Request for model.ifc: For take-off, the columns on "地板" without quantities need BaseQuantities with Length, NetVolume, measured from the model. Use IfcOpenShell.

First a look at what the model holds.

```python
import ifcopenshell
import ifcopenshell.util.element
import ifcopenshell.util.unit

model = ifcopenshell.open("model.ifc")
print(model.schema)
for unit_type in ("LENGTHUNIT", "AREAUNIT", "VOLUMEUNIT"):
    print(unit_type, ifcopenshell.util.unit.calculate_unit_scale(model, unit_type))
storey = next(s for s in model.by_type("IfcBuildingStorey") if s.Name == "地板")
columns = [e for e in ifcopenshell.util.element.get_decomposition(storey) if e.is_a("IfcColumn")]
for e in sorted(columns, key=lambda e: e.id()):
    print(e.id(), e.is_a(), e.Name, list(ifcopenshell.util.element.get_psets(e, qtos_only=True)), sep=" | ")
```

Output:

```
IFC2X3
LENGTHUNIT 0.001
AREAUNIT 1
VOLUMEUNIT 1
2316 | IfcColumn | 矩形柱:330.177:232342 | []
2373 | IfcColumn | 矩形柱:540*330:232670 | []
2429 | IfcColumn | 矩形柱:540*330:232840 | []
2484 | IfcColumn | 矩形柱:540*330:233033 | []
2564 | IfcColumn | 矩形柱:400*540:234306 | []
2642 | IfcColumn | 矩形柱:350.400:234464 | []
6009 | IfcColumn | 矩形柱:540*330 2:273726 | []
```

```python
import ifcopenshell
import ifcopenshell.api.pset
import ifcopenshell.geom
import ifcopenshell.util.element
import ifcopenshell.util.shape
import ifcopenshell.util.unit

model = ifcopenshell.open("model.ifc")
unit_scale = ifcopenshell.util.unit.calculate_unit_scale(model)
volume_scale = ifcopenshell.util.unit.calculate_unit_scale(model, "VOLUMEUNIT")
settings = ifcopenshell.geom.settings()

storey = next(s for s in model.by_type("IfcBuildingStorey") if s.Name == "地板")
columns = [e for e in ifcopenshell.util.element.get_decomposition(storey) if e.is_a("IfcColumn")]

for e in sorted(columns, key=lambda e: e.id()):
    if ifcopenshell.util.element.get_psets(e, qtos_only=True, should_inherit=False):
        continue
    # Geometry comes back in metres, in the element's own axes.
    shape = ifcopenshell.geom.create_shape(settings, e)
    values = {
        "Length": ifcopenshell.util.shape.get_z(shape.geometry) / unit_scale,
        "NetVolume": ifcopenshell.util.shape.get_volume(shape.geometry) / volume_scale,
    }
    qto = ifcopenshell.api.pset.add_qto(model, product=e, name="BaseQuantities")
    ifcopenshell.api.pset.edit_qto(model, qto=qto, properties=values)
    print(e.id(), {k: round(v, 3) for k, v in values.items()})

model.write("model_v2.ifc")
```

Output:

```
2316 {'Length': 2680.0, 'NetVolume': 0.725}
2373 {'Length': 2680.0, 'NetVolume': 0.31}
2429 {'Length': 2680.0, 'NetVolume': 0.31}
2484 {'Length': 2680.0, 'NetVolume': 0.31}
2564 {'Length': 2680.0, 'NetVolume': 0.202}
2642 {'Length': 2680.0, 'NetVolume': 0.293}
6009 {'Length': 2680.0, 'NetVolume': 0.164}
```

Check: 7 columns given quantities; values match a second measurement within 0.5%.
